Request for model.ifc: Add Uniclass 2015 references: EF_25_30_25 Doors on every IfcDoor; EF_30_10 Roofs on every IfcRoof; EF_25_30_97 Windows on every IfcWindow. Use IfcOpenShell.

First a look at what the model holds.

```python
import ifcopenshell

model = ifcopenshell.open("model.ifc")
print(model.schema)
print("classifications:", [c.Name for c in model.by_type("IfcClassification")])
for ifc_class in ("IfcDoor", "IfcRoof", "IfcStair", "IfcWall", "IfcWindow"):
    print(ifc_class, len(model.by_type(ifc_class)))
```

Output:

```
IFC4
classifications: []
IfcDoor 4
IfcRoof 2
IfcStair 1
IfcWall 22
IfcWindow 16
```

```python
import ifcopenshell
import ifcopenshell.api.classification

model = ifcopenshell.open("model.ifc")

system = ifcopenshell.api.classification.add_classification(model, classification="Uniclass 2015")

codes = {
    "IfcDoor": ("EF_25_30_25", "Doors"),
    "IfcRoof": ("EF_30_10", "Roofs"),
    "IfcWindow": ("EF_25_30_97", "Windows"),
}
for ifc_class, (code, name) in codes.items():
    products = model.by_type(ifc_class)
    ifcopenshell.api.classification.add_reference(
        model, products=products, classification=system, identification=code, name=name
    )
    print(code, len(products))

model.write("model-out.ifc")
```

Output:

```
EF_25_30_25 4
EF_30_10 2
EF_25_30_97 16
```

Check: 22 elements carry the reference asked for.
